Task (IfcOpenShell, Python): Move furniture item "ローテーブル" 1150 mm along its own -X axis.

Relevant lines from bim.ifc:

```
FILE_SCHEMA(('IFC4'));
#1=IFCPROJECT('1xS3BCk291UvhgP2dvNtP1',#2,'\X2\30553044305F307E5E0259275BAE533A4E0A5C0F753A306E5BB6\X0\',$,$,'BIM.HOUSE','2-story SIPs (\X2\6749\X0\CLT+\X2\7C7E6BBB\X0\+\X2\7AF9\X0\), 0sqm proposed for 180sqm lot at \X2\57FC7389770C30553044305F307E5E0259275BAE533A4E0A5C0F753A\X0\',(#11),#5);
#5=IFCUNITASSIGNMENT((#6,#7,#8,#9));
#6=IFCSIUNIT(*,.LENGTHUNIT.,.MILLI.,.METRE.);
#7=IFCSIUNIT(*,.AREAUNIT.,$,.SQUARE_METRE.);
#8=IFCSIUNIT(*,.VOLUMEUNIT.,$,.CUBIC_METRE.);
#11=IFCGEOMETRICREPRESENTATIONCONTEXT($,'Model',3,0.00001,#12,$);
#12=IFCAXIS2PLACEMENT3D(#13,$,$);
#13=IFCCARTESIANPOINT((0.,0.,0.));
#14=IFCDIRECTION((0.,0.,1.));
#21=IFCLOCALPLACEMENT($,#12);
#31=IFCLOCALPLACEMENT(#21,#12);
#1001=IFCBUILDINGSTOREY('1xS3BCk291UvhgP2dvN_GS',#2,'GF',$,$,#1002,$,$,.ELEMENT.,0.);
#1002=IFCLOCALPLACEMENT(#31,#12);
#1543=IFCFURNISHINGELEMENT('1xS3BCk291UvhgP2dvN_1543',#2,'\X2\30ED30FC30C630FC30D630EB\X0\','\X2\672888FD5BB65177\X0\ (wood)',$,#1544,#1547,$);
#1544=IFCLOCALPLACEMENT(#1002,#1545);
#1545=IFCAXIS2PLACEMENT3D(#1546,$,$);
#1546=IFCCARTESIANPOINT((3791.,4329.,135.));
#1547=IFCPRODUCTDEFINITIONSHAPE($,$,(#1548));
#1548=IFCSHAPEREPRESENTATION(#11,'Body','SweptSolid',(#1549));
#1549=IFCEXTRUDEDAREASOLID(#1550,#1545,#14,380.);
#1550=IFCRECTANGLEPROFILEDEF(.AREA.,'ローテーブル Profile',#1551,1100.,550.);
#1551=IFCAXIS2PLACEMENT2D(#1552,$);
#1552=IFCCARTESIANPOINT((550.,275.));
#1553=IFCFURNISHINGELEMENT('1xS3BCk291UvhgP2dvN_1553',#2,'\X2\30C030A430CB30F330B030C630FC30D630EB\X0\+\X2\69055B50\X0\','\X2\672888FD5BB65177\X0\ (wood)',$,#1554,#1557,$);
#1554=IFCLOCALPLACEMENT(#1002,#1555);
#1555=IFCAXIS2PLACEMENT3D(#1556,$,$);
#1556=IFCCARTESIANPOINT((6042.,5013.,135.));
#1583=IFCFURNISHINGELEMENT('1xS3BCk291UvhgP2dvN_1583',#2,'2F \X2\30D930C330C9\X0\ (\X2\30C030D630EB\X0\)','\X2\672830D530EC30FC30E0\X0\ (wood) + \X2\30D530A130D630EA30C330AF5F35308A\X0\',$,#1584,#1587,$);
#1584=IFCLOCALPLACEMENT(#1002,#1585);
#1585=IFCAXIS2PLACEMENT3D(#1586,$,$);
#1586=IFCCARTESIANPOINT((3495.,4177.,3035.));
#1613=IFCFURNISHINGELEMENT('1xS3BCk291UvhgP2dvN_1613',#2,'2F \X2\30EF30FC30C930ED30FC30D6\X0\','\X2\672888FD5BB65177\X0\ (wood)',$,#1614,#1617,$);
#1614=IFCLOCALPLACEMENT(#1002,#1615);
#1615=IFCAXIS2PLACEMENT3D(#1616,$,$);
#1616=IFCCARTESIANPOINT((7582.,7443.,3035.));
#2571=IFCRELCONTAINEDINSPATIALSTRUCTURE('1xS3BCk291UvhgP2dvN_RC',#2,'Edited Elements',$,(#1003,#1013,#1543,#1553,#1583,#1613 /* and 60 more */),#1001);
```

```python
import ifcopenshell
import ifcopenshell.api.geometry
import ifcopenshell.util.placement
import ifcopenshell.util.unit

model = ifcopenshell.open("bim.ifc")
unit_scale = ifcopenshell.util.unit.calculate_unit_scale(model)

item = model.by_guid("1xS3BCk291UvhgP2dvN_1543")
matrix = ifcopenshell.util.placement.get_local_placement(item.ObjectPlacement)
matrix[:3, 3] -= matrix[:3, 0] * 1.15 / unit_scale
ifcopenshell.api.geometry.edit_object_placement(model, product=item, matrix=matrix, is_si=False)

print(ifcopenshell.util.placement.get_local_placement(item.ObjectPlacement).round(3) + 0.0)

model.write("bim_v2.ifc")
```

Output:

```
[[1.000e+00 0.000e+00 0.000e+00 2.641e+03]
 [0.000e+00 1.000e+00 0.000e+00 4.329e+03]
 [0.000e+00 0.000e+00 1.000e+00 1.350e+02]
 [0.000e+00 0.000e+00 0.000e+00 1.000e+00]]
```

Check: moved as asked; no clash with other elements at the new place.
